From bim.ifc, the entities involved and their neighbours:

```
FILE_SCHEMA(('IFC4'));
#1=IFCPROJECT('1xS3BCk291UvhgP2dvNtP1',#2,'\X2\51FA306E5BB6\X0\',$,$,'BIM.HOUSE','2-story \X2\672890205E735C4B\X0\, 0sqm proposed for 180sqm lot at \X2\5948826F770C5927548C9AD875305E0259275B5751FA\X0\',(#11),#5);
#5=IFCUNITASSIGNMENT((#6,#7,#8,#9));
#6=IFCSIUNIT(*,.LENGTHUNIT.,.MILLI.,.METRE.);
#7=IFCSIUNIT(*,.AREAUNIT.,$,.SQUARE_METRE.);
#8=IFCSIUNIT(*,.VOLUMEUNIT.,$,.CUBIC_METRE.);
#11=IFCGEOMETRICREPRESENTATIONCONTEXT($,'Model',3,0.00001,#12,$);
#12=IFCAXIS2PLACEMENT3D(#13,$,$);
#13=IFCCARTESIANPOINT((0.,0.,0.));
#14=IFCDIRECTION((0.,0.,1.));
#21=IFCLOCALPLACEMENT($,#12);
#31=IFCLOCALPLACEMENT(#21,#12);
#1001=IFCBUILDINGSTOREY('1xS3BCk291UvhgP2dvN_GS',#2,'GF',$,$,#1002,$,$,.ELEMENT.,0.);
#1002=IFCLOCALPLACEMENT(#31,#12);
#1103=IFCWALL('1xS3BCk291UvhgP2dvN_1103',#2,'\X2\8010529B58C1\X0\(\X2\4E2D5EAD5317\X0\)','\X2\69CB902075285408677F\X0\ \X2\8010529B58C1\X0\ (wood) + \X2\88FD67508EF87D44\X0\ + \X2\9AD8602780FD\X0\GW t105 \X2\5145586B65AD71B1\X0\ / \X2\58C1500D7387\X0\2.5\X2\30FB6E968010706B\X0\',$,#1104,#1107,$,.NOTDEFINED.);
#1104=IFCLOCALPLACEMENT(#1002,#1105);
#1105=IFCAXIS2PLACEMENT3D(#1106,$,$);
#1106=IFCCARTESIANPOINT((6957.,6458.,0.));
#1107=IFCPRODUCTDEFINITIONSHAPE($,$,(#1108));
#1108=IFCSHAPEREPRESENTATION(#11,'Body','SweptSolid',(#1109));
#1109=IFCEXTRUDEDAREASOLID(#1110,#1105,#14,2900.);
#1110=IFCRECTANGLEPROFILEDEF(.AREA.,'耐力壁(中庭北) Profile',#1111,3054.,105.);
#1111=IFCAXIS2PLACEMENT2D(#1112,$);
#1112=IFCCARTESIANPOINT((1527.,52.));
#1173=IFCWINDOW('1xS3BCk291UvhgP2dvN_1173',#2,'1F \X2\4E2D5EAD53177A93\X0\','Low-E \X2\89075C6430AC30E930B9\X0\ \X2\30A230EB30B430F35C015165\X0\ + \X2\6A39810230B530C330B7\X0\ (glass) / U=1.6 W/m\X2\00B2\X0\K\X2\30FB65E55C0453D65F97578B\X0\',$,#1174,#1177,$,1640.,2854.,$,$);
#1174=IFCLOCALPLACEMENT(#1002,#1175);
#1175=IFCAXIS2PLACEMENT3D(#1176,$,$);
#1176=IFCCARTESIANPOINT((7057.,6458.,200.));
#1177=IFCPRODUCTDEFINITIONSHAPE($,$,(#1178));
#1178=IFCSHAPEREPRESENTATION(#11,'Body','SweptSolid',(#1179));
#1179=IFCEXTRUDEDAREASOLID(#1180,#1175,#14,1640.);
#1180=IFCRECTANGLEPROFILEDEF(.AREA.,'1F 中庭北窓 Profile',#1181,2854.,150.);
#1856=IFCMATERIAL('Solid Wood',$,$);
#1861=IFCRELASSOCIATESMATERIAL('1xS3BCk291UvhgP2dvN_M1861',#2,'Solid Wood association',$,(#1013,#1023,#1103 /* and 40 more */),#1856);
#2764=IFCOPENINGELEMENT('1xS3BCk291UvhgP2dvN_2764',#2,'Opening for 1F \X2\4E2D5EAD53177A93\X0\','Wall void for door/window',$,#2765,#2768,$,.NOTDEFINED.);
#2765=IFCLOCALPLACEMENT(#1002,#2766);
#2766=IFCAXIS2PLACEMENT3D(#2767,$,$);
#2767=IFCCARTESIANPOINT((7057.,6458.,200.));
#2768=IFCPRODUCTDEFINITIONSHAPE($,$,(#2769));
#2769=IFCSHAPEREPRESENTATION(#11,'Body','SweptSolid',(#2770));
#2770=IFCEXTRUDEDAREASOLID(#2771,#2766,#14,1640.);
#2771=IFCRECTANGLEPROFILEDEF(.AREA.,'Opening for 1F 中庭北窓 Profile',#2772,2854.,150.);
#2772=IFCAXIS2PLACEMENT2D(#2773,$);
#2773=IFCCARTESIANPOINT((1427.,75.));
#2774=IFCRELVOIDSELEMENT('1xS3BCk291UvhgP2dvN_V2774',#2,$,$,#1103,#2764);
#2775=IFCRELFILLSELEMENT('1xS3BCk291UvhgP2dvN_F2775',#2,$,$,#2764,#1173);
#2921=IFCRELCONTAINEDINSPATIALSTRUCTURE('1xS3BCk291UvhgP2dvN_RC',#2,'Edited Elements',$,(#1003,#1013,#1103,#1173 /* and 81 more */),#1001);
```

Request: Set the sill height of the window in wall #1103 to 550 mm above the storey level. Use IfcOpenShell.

```python
import numpy as np
import ifcopenshell
import ifcopenshell.api.geometry
import ifcopenshell.geom
import ifcopenshell.util.element
import ifcopenshell.util.placement
import ifcopenshell.util.shape
import ifcopenshell.util.unit

model = ifcopenshell.open("bim.ifc")
unit_scale = ifcopenshell.util.unit.calculate_unit_scale(model)

window = model.by_guid("1xS3BCk291UvhgP2dvN_1173")
opening = window.FillsVoids[0].RelatingOpeningElement
storey = ifcopenshell.util.element.get_container(window, ifc_class="IfcBuildingStorey")
level = ifcopenshell.util.placement.get_local_placement(storey.ObjectPlacement)[2, 3]

# The opening's origin need not be at the sill, so measure its lowest point.
shape = ifcopenshell.geom.create_shape(ifcopenshell.geom.settings(), opening)
bottom = ifcopenshell.util.shape.get_shape_bottom_elevation(shape, shape.geometry) / unit_scale
dz = level + 0.55 / unit_scale - bottom

shift = np.array([0.0, 0.0, dz])
# The window is not placed relative to its opening, so move both.
for product in (opening, window):
    matrix = ifcopenshell.util.placement.get_local_placement(product.ObjectPlacement)
    matrix[:3, 3] += shift
    ifcopenshell.api.geometry.edit_object_placement(model, product=product, matrix=matrix, is_si=False)

print(f"moved by {dz * unit_scale:+.3f} m")

model.write("bim_rev.ifc")
```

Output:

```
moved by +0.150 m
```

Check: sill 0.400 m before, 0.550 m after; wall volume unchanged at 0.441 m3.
